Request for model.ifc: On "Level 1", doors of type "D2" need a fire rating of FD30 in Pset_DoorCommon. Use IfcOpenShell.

First a look at what the model holds.

```python
import ifcopenshell
import ifcopenshell.util.element

model = ifcopenshell.open("model.ifc")
print(model.schema)
storey = next(s for s in model.by_type("IfcBuildingStorey") if s.Name == "Level 1")
doors = [e for e in ifcopenshell.util.element.get_decomposition(storey) if e.is_a("IfcDoor")]
seen = {}
for e in doors:
    element_type = ifcopenshell.util.element.get_type(e)
    key = (element_type.Name if element_type != e and element_type else None, ifcopenshell.util.element.get_pset(e, "Pset_DoorCommon", "FireRating"))
    seen[key] = seen.get(key, 0) + 1
for (name, value), count in sorted(seen.items(), key=str):
    print(count, "x", name, "|", value)
```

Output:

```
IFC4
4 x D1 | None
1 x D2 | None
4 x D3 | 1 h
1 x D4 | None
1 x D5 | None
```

```python
import ifcopenshell
import ifcopenshell.api.pset
import ifcopenshell.util.element

model = ifcopenshell.open("model.ifc")

storey = next(s for s in model.by_type("IfcBuildingStorey") if s.Name == "Level 1")
doors = [e for e in ifcopenshell.util.element.get_decomposition(storey) if e.is_a("IfcDoor")]

count = 0
for e in doors:
    element_type = ifcopenshell.util.element.get_type(e)
    if element_type in (None, e) or element_type.Name != "D2":
        continue
    # add_pset returns the element's existing set when there is one.
    pset = ifcopenshell.api.pset.add_pset(model, product=e, name="Pset_DoorCommon")
    ifcopenshell.api.pset.edit_pset(model, pset=pset, properties={"FireRating": "FD30"})
    count += 1

print(count, "doors updated")

model.write("model_v2.ifc")
```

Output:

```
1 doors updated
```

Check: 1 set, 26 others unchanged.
